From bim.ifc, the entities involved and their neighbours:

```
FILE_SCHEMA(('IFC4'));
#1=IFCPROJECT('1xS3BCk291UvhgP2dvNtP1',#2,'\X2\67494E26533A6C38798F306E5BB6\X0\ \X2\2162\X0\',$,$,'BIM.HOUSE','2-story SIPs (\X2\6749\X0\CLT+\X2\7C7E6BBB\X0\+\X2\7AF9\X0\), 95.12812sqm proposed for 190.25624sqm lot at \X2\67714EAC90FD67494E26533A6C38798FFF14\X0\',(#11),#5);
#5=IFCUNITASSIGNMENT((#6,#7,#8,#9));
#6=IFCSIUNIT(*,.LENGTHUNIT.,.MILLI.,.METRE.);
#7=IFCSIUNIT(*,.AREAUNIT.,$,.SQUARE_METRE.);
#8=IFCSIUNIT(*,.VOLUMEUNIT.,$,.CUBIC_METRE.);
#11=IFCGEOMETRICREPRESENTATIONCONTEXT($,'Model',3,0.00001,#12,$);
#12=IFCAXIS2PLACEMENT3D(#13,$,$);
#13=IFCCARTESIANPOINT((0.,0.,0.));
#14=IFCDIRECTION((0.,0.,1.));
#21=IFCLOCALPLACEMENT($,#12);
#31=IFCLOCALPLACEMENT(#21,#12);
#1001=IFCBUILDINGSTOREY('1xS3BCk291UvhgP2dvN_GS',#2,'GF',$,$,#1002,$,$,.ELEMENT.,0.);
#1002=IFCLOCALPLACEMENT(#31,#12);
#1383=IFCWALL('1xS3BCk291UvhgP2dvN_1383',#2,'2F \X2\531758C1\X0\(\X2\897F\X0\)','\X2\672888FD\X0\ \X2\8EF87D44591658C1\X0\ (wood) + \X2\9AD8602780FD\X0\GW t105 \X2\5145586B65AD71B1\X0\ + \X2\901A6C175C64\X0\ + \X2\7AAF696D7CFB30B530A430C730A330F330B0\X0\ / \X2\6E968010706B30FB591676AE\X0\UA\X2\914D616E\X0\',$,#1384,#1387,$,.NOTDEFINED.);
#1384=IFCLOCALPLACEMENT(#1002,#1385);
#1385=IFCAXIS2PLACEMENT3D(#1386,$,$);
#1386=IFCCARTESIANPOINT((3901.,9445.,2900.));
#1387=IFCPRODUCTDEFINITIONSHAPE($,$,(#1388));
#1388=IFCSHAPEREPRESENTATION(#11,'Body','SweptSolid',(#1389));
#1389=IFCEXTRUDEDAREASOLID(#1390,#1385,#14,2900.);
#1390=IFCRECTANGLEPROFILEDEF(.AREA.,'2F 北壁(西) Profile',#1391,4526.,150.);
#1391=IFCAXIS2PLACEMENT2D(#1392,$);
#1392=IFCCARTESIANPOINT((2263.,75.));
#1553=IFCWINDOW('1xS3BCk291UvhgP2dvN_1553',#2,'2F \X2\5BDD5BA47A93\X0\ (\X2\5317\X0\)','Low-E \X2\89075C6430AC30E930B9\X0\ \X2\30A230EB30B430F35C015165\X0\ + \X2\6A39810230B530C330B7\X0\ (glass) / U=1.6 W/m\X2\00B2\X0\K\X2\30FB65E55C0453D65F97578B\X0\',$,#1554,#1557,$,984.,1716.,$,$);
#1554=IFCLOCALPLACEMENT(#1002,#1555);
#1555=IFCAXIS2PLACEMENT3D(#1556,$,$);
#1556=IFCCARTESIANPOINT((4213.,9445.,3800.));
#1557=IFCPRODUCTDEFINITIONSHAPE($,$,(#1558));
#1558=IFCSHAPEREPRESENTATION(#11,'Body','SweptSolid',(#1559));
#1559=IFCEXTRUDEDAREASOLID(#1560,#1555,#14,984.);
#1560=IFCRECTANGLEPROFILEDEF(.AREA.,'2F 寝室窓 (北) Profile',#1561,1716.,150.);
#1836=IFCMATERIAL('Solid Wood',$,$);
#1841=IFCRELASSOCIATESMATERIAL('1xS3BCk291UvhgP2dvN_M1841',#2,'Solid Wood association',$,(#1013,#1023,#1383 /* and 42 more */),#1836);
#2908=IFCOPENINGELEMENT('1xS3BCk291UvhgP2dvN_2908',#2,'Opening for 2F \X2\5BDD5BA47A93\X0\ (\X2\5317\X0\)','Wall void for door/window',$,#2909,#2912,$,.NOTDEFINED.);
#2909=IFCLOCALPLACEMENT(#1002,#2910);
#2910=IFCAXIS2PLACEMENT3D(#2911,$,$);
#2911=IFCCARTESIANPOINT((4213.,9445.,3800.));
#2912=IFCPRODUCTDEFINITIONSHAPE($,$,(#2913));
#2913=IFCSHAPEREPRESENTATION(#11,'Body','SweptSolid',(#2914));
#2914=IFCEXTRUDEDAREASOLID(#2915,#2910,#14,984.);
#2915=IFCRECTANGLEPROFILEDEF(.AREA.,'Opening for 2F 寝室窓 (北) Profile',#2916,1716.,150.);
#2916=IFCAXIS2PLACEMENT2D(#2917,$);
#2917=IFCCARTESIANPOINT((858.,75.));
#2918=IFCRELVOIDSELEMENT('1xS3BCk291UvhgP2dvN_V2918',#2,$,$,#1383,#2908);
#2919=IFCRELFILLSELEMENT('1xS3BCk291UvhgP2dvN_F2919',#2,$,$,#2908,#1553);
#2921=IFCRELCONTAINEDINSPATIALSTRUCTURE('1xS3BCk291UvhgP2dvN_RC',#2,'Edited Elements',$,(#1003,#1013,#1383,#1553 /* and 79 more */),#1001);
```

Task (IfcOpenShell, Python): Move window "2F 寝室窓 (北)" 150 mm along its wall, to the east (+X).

```python
import ifcopenshell
import ifcopenshell.api.geometry
import ifcopenshell.util.placement

model = ifcopenshell.open("bim.ifc")

window = model.by_guid("1xS3BCk291UvhgP2dvN_1553")
opening = window.FillsVoids[0].RelatingOpeningElement
wall = opening.VoidsElements[0].RelatingBuildingElement

wall_matrix = ifcopenshell.util.placement.get_local_placement(wall.ObjectPlacement)
shift = wall_matrix[:3, 0] * 150.0
before = ifcopenshell.util.placement.get_local_placement(window.ObjectPlacement)[:3, 3].copy()

# The window is not placed relative to its opening, so move both.
for product in (opening, window):
    matrix = ifcopenshell.util.placement.get_local_placement(product.ObjectPlacement)
    matrix[:3, 3] += shift
    ifcopenshell.api.geometry.edit_object_placement(model, product=product, matrix=matrix, is_si=False)

after = ifcopenshell.util.placement.get_local_placement(window.ObjectPlacement)[:3, 3]
print("window moved by", (after - before).round(3) + 0.0)

model.write("bim_rev.ifc")
```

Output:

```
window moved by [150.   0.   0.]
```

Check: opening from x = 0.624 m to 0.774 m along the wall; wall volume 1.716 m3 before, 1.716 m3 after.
